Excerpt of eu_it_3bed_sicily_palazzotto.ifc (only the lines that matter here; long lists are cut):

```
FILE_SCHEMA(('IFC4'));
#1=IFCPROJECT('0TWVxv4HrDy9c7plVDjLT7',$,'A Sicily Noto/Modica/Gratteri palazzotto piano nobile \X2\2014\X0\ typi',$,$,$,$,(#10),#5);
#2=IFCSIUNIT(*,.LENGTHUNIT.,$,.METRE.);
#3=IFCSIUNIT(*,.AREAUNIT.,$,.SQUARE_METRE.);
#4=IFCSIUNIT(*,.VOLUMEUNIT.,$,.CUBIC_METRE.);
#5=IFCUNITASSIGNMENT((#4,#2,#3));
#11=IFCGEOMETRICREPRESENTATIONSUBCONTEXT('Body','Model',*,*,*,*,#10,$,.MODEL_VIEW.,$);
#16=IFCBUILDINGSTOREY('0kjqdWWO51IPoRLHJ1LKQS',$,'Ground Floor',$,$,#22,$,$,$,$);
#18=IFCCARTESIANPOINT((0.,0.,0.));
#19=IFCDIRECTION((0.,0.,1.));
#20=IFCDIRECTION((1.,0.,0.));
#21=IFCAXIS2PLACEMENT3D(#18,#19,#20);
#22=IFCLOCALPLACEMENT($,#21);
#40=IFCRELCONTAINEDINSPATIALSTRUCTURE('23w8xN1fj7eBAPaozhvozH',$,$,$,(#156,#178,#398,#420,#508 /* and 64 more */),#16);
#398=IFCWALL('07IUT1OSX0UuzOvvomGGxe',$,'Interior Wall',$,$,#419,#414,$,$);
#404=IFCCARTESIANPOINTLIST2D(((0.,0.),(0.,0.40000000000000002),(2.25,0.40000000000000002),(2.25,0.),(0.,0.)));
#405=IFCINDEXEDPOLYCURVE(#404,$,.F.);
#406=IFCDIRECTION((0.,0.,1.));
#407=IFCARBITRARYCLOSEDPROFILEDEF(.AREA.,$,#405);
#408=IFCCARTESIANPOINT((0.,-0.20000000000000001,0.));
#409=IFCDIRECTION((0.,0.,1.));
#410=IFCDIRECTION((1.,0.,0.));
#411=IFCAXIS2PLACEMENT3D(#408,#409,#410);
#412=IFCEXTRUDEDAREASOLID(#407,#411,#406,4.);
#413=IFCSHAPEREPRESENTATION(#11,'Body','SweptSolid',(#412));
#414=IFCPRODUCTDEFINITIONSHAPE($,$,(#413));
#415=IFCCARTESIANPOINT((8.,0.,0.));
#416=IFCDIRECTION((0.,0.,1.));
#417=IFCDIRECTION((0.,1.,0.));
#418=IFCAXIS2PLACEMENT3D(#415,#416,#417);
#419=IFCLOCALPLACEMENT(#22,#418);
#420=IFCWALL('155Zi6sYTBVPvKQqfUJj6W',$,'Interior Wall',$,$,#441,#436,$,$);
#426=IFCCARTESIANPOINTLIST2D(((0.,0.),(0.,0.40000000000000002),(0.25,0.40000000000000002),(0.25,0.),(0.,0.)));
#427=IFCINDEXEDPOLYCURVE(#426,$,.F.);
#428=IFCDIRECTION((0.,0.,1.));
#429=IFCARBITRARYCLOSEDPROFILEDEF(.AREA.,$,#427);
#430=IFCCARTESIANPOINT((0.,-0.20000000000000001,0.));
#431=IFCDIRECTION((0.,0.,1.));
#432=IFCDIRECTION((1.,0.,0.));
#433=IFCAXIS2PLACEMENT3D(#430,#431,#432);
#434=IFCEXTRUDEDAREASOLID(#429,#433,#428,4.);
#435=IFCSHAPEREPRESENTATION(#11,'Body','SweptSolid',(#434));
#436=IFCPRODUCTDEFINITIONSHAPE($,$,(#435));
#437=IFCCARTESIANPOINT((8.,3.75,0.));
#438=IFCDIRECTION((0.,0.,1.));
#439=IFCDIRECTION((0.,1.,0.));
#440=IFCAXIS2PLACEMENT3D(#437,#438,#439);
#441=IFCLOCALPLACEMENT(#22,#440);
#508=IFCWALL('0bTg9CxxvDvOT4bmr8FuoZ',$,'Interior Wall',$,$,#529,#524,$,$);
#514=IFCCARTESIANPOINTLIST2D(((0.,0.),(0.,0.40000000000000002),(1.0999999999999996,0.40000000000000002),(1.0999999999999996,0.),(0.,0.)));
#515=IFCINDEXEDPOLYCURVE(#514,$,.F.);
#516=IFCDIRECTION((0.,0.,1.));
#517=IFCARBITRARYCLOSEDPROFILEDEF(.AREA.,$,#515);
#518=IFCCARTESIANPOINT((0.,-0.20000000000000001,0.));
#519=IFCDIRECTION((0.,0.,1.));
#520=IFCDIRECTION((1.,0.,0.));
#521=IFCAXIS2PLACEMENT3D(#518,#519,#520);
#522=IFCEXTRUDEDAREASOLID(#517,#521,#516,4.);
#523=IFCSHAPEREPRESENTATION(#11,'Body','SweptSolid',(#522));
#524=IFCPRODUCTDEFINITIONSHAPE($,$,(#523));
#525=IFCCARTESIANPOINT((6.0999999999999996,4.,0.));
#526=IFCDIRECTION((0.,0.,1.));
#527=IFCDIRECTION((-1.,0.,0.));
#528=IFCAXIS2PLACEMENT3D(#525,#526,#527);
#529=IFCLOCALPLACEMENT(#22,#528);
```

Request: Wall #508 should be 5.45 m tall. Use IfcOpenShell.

```python
import ifcopenshell
import ifcopenshell.geom
import ifcopenshell.util.representation
import ifcopenshell.util.shape
import ifcopenshell.util.unit

model = ifcopenshell.open("eu_it_3bed_sicily_palazzotto.ifc")
unit_scale = ifcopenshell.util.unit.calculate_unit_scale(model)
settings = ifcopenshell.geom.settings()


def volume(element):
    """Net volume in cubic metres, openings subtracted."""
    shape = ifcopenshell.geom.create_shape(settings, element)
    return ifcopenshell.util.shape.get_volume(shape.geometry)


wall = model.by_guid("0bTg9CxxvDvOT4bmr8FuoZ")
before = volume(wall)

body = ifcopenshell.util.representation.get_representation(wall, "Model", "Body")
solid = body.Items[0]
old_height = solid.Depth
solid.Depth = 5.45 / unit_scale
after = volume(wall)

print(f"height {old_height:g} -> {solid.Depth:g}, volume {before:.3f} -> {after:.3f} m3")

model.write("eu_it_3bed_sicily_palazzotto_v2.ifc")
```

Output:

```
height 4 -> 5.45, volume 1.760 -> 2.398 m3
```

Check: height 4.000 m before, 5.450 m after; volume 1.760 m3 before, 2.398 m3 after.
